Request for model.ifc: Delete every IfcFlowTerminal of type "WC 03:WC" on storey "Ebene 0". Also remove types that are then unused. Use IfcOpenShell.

First a look at what the model holds.

```python
import ifcopenshell
import ifcopenshell.util.element

model = ifcopenshell.open("model.ifc")
print(model.schema)
storey = next(s for s in model.by_type("IfcBuildingStorey") if s.Name == "Ebene 0")
terminals = [e for e in ifcopenshell.util.element.get_decomposition(storey) if e.is_a("IfcFlowTerminal")]
seen = {}
for e in terminals:
    element_type = ifcopenshell.util.element.get_type(e)
    name = element_type.Name if element_type not in (None, e) else None
    seen[name] = seen.get(name, 0) + 1
for name, count in sorted(seen.items(), key=str):
    print(count, "x", name)
```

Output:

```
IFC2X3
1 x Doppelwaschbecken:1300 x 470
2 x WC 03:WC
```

```python
import ifcopenshell
import ifcopenshell.api.root
import ifcopenshell.util.element

model = ifcopenshell.open("model.ifc")

storey = next(s for s in model.by_type("IfcBuildingStorey") if s.Name == "Ebene 0")
terminals = [e for e in ifcopenshell.util.element.get_decomposition(storey) if e.is_a("IfcFlowTerminal")]
targets = [e for e in terminals if (t := ifcopenshell.util.element.get_type(e)) not in (None, e) and t.Name == "WC 03:WC"]
types = {ifcopenshell.util.element.get_type(e) for e in targets} - {None, *targets}

for e in targets:
    ifcopenshell.api.root.remove_product(model, product=e)
print(len(targets), "removed")

unused = [t for t in types if not ifcopenshell.util.element.get_types(t)]
for t in unused:
    ifcopenshell.api.root.remove_product(model, product=t)
print(len(unused), "unused types removed")

model.write("model_v2.ifc")
```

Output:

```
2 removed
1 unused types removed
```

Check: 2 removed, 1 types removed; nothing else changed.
